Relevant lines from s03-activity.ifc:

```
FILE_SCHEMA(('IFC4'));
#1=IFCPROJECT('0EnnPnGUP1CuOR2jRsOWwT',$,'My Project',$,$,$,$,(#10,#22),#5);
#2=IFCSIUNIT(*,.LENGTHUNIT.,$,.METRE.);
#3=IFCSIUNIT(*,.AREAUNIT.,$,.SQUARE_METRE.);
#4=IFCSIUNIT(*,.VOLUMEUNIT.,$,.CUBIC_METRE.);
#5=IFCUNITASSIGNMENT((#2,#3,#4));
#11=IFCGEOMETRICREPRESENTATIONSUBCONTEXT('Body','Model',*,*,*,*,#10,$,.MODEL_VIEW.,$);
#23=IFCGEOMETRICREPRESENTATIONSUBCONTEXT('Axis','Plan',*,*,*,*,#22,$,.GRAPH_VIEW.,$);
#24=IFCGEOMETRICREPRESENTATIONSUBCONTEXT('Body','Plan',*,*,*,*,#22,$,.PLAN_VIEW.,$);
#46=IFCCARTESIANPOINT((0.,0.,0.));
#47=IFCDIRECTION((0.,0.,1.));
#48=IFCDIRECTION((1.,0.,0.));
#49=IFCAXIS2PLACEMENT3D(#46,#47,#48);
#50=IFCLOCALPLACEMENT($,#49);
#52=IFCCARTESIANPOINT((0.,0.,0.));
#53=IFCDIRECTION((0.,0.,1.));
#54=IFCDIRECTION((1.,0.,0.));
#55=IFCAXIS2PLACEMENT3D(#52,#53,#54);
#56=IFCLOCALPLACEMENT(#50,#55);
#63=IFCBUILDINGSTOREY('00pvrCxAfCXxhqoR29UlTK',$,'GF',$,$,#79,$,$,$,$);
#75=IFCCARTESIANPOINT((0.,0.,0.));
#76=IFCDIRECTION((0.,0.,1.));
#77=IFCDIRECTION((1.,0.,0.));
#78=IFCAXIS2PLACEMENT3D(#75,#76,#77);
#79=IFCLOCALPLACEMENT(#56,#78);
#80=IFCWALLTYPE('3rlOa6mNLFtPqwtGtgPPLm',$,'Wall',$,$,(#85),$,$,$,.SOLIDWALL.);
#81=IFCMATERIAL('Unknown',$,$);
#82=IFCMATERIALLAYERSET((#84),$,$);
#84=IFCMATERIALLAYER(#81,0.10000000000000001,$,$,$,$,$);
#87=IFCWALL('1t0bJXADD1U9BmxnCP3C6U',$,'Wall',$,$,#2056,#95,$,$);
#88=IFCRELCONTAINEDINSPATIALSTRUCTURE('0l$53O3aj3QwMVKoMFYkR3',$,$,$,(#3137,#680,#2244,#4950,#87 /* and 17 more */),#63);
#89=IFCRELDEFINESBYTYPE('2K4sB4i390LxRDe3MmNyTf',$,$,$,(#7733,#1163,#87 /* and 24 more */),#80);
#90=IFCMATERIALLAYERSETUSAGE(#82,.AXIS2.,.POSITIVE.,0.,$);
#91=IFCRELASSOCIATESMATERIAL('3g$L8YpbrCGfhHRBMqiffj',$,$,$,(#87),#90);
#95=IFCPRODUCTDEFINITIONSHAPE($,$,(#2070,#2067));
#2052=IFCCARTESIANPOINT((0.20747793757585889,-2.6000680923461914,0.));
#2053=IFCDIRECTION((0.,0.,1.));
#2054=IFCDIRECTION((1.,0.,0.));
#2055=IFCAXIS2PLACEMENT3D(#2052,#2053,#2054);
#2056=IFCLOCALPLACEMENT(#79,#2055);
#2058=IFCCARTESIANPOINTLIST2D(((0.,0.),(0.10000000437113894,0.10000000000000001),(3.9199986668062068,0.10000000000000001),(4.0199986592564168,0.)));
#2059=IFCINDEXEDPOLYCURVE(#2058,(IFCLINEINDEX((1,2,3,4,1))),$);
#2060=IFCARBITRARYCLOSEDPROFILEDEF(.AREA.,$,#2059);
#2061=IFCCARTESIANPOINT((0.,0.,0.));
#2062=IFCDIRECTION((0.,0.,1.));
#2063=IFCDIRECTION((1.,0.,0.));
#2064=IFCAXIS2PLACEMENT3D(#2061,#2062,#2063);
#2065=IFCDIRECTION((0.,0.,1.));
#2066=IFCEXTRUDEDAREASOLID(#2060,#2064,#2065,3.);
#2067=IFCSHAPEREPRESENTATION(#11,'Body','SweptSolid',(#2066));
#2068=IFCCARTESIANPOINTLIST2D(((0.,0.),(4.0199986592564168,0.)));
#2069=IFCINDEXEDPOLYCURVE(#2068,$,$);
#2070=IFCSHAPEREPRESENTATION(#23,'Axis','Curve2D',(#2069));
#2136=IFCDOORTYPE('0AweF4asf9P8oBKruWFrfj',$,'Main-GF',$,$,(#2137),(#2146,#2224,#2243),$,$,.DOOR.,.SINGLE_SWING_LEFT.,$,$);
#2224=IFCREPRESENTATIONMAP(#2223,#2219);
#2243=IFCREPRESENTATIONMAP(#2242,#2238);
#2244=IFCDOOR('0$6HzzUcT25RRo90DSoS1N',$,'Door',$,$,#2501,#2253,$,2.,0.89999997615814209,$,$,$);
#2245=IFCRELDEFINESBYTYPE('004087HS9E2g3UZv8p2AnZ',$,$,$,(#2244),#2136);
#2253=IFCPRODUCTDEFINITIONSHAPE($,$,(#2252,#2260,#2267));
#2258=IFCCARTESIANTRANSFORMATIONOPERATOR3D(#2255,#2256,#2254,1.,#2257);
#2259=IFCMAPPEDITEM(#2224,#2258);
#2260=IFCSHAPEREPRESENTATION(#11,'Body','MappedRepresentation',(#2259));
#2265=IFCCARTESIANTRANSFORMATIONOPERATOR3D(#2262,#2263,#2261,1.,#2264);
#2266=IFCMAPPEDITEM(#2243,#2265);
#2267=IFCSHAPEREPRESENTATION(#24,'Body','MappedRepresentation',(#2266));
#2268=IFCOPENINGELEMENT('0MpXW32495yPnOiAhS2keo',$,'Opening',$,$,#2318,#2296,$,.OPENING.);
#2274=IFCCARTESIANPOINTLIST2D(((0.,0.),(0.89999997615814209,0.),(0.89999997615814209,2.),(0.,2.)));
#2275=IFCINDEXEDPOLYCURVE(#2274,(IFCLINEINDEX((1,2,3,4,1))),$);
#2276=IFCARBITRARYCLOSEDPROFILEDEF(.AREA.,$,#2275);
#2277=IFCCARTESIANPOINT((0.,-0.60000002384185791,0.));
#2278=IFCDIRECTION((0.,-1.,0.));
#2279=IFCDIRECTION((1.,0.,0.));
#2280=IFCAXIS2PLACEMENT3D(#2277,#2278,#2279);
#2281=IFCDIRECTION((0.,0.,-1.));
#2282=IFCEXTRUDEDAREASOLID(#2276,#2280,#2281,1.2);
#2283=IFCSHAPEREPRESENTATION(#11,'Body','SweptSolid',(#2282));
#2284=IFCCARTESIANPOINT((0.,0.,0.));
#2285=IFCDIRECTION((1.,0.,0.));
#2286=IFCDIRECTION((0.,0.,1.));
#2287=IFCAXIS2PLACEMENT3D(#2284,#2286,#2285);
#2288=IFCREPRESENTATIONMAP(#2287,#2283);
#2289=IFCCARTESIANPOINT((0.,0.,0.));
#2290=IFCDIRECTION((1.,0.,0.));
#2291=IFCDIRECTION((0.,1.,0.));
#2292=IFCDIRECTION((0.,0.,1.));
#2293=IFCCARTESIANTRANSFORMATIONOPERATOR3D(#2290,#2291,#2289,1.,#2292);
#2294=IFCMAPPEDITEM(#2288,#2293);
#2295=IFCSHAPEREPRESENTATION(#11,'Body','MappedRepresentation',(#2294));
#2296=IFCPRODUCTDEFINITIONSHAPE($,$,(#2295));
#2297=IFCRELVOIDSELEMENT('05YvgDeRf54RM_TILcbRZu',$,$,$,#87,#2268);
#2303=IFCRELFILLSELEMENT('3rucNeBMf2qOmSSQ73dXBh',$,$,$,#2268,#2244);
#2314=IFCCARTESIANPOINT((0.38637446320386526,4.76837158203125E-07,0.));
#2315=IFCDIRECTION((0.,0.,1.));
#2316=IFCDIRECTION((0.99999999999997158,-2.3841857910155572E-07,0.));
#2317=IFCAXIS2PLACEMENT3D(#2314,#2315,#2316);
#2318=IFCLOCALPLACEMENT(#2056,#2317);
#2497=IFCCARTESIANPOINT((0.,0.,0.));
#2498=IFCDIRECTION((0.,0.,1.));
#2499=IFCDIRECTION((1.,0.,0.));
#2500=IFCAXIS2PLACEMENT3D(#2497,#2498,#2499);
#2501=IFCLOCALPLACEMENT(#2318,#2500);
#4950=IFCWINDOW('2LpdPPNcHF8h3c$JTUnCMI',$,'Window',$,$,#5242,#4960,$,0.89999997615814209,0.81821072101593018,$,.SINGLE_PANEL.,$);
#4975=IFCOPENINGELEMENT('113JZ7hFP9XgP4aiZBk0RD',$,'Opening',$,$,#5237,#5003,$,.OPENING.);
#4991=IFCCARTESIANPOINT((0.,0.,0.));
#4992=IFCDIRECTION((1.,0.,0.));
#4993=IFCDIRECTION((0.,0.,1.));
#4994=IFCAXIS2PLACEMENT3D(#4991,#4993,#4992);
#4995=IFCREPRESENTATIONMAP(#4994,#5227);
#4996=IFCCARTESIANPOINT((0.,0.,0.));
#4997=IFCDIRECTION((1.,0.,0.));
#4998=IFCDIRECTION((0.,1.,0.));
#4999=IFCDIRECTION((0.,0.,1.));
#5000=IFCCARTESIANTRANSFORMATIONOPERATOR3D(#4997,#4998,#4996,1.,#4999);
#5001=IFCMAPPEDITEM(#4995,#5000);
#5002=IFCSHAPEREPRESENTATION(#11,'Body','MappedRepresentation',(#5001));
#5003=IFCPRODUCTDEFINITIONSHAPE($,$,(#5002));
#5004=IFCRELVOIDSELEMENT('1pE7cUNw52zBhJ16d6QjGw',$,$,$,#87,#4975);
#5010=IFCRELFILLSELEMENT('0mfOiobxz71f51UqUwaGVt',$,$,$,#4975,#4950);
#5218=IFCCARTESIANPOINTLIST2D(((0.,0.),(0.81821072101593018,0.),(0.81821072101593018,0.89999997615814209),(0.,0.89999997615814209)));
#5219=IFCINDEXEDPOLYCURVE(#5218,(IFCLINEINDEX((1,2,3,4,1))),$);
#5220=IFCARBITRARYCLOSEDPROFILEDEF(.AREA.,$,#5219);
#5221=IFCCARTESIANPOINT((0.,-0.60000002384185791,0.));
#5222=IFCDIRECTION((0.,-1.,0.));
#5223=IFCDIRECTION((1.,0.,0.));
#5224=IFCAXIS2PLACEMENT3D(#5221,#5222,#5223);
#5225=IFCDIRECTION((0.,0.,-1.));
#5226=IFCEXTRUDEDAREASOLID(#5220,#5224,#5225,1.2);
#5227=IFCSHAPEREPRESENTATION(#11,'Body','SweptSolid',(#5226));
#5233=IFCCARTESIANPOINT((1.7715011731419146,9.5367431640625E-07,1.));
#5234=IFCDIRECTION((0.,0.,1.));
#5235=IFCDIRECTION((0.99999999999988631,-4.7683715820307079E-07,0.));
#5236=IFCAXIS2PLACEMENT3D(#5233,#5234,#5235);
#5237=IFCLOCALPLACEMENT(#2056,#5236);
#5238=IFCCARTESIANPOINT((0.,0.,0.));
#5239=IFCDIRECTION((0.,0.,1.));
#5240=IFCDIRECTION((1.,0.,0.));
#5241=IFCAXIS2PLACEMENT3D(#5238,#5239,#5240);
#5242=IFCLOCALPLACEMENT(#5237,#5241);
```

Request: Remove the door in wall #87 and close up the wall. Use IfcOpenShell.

```python
import ifcopenshell
import ifcopenshell.api.feature
import ifcopenshell.api.root
import ifcopenshell.geom
import ifcopenshell.util.shape

model = ifcopenshell.open("s03-activity.ifc")
settings = ifcopenshell.geom.settings()


def volume(element):
    """Net volume in cubic metres, openings subtracted."""
    shape = ifcopenshell.geom.create_shape(settings, element)
    return ifcopenshell.util.shape.get_volume(shape.geometry)


door = model.by_guid("0$6HzzUcT25RRo90DSoS1N")
opening = door.FillsVoids[0].RelatingOpeningElement
wall = opening.VoidsElements[0].RelatingBuildingElement
before = volume(wall)

ifcopenshell.api.root.remove_product(model, product=door)
ifcopenshell.api.feature.remove_feature(model, feature=opening)

after = volume(wall)

print(f"wall volume {before:.3f} -> {after:.3f} m3")

model.write("s03-activity_updated.ifc")
```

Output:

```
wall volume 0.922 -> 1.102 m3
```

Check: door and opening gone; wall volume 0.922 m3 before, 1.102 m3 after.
